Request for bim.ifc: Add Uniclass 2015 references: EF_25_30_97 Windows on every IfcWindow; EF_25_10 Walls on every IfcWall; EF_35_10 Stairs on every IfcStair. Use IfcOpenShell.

First a look at what the model holds.

```python
import ifcopenshell

model = ifcopenshell.open("bim.ifc")
print(model.schema)
print("classifications:", [c.Name for c in model.by_type("IfcClassification")])
for ifc_class in ("IfcDoor", "IfcRoof", "IfcStair", "IfcWall", "IfcWindow"):
    print(ifc_class, len(model.by_type(ifc_class)))
```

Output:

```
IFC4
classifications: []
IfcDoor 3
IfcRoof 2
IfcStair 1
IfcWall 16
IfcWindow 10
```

```python
import ifcopenshell
import ifcopenshell.api.classification

model = ifcopenshell.open("bim.ifc")

system = ifcopenshell.api.classification.add_classification(model, classification="Uniclass 2015")

codes = {
    "IfcWindow": ("EF_25_30_97", "Windows"),
    "IfcWall": ("EF_25_10", "Walls"),
    "IfcStair": ("EF_35_10", "Stairs"),
}
for ifc_class, (code, name) in codes.items():
    products = model.by_type(ifc_class)
    ifcopenshell.api.classification.add_reference(
        model, products=products, classification=system, identification=code, name=name
    )
    print(code, len(products))

model.write("bim_edited.ifc")
```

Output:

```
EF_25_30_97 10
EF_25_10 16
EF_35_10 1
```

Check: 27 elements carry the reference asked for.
